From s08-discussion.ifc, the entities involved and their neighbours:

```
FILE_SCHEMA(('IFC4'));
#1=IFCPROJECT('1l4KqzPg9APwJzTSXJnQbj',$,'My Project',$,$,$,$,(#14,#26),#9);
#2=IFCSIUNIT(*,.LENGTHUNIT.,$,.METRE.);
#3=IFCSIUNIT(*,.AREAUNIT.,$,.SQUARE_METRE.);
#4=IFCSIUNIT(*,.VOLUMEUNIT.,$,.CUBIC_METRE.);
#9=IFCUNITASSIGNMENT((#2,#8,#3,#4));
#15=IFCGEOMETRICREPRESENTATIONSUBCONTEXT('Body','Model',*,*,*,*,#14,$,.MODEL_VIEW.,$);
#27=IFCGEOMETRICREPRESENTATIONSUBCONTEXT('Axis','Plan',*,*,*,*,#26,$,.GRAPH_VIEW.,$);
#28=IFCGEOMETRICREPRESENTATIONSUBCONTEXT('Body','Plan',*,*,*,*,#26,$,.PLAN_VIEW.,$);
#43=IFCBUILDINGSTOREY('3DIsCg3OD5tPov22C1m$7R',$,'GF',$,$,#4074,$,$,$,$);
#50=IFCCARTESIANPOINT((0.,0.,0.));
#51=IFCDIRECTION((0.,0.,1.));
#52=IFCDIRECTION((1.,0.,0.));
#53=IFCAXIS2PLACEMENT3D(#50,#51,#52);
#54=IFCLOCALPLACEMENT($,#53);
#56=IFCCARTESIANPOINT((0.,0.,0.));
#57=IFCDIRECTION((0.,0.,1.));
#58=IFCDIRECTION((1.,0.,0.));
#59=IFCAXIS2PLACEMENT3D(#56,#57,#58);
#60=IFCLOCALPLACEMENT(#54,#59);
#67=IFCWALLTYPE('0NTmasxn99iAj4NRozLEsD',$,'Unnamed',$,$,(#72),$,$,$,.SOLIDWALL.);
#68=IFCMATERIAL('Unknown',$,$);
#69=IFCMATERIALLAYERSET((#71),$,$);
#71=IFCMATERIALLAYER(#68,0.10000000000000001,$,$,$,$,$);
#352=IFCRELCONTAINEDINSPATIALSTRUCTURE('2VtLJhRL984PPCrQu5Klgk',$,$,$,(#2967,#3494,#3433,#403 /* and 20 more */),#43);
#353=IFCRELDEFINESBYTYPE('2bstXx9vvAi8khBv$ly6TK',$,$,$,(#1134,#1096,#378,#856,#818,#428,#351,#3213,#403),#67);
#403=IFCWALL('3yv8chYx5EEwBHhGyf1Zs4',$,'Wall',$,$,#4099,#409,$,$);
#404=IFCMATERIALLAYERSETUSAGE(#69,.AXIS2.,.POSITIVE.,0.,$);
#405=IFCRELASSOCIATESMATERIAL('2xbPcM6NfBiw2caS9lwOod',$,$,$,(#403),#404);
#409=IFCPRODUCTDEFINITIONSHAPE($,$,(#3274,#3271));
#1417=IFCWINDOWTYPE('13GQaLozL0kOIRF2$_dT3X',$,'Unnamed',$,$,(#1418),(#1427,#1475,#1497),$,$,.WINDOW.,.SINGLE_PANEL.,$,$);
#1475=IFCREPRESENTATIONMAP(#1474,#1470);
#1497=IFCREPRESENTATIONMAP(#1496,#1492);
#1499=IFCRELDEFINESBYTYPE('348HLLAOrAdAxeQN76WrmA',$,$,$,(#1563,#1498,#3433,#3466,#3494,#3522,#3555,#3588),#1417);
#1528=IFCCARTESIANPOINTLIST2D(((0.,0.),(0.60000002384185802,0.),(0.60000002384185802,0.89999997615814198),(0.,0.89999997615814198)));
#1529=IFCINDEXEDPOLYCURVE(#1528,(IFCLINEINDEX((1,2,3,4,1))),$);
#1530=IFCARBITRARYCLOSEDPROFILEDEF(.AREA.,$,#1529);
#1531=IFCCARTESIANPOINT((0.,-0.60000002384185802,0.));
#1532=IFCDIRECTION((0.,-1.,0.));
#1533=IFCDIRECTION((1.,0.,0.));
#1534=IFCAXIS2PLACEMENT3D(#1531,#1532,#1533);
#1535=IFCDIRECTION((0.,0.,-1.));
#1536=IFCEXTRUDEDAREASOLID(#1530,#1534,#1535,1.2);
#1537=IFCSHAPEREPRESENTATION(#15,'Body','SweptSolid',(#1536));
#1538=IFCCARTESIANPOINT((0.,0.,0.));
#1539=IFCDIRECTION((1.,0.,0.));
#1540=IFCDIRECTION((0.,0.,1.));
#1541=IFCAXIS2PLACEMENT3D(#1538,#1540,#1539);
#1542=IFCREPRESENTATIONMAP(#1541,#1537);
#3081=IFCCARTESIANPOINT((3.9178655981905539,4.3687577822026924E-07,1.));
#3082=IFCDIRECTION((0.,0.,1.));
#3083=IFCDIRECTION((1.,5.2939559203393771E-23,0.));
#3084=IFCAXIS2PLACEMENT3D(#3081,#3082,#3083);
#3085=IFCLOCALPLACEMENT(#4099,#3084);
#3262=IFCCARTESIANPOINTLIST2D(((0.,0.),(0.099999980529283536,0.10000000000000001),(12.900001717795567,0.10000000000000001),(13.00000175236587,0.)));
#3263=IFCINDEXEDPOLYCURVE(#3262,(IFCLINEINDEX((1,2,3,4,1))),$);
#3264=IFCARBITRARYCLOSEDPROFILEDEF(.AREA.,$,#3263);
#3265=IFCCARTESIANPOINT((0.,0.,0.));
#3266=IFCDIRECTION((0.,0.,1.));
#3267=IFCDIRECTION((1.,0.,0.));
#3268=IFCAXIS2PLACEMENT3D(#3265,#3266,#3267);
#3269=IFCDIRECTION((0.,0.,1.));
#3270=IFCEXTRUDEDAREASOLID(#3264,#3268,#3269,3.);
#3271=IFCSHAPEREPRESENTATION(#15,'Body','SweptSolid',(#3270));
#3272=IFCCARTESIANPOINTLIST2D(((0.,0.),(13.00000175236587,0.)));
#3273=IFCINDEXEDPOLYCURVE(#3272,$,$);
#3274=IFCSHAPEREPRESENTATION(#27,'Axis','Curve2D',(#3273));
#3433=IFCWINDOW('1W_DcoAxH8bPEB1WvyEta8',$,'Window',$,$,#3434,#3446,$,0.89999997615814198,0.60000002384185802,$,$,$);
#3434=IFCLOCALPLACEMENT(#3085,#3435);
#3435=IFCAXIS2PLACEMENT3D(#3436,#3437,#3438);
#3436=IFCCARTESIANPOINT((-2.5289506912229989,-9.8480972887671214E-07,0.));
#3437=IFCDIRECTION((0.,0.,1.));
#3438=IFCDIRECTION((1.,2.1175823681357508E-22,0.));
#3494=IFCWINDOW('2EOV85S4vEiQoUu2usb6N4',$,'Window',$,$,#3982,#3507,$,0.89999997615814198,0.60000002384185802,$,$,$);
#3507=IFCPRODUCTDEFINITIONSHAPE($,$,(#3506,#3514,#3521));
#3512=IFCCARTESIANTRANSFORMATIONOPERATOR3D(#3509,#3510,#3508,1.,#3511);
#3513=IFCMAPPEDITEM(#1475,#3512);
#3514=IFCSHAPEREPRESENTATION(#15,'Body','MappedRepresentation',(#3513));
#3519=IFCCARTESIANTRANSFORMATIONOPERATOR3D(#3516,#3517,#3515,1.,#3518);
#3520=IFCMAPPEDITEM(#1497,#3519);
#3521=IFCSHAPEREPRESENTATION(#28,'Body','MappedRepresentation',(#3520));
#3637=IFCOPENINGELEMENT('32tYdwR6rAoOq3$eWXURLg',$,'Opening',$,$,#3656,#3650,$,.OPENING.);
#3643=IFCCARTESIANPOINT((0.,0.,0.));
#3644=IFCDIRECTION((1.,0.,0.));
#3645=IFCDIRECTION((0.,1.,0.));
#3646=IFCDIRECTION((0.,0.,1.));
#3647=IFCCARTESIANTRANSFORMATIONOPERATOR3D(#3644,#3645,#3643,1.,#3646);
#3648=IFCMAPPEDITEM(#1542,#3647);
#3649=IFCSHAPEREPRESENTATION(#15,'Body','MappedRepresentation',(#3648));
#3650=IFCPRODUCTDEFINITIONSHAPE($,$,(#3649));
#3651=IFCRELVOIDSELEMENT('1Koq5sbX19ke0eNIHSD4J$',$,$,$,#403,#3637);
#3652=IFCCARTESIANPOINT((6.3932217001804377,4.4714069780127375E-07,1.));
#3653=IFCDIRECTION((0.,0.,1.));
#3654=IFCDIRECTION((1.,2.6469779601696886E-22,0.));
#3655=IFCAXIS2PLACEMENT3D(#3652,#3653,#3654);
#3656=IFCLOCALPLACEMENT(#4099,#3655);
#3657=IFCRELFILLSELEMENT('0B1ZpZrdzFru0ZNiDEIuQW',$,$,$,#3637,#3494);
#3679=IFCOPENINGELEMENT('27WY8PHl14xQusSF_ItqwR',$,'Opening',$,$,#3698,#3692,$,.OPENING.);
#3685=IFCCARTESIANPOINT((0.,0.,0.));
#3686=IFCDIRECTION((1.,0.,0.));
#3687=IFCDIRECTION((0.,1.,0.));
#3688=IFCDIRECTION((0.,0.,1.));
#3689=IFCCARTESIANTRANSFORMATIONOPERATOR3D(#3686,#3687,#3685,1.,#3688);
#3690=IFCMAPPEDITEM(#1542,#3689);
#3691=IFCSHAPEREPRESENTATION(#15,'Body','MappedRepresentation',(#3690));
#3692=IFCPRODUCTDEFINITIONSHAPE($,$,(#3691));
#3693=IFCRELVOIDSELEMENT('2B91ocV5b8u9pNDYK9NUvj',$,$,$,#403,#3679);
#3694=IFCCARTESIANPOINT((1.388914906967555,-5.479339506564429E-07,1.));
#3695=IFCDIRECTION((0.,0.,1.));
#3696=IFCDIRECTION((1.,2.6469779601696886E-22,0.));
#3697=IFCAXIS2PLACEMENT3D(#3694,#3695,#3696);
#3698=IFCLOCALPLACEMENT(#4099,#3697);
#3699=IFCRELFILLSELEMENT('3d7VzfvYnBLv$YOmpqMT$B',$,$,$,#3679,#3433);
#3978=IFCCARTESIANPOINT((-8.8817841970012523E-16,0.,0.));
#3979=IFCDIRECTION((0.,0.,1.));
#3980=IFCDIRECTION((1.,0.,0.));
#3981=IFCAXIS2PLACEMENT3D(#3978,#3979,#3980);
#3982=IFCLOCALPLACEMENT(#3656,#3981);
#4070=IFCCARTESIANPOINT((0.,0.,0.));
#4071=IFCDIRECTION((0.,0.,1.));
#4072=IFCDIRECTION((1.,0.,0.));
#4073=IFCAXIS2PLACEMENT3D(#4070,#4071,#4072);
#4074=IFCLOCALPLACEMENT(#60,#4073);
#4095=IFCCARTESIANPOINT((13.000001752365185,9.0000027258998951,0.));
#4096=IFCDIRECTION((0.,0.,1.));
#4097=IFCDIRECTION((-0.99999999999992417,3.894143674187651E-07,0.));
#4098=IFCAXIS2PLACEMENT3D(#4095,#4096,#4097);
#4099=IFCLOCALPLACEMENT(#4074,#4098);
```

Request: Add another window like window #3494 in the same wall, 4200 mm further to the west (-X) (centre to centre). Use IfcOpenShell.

```python
import ifcopenshell
import ifcopenshell.api.feature
import ifcopenshell.api.geometry
import ifcopenshell.api.root
import ifcopenshell.geom
import ifcopenshell.util.element
import ifcopenshell.util.placement
import ifcopenshell.util.shape
import ifcopenshell.util.unit

model = ifcopenshell.open("s08-discussion.ifc")
unit_scale = ifcopenshell.util.unit.calculate_unit_scale(model)
settings = ifcopenshell.geom.settings()


def volume(element):
    """Net volume in cubic metres, openings subtracted."""
    shape = ifcopenshell.geom.create_shape(settings, element)
    return ifcopenshell.util.shape.get_volume(shape.geometry)


window = model.by_id(3494)
opening = window.FillsVoids[0].RelatingOpeningElement
wall = opening.VoidsElements[0].RelatingBuildingElement
before = volume(wall)
shift = ifcopenshell.util.placement.get_local_placement(wall.ObjectPlacement)[:3, 0] * 4.2 / unit_scale

# copy_class copies the void relationship, type, container and properties, but no geometry.
new_opening = ifcopenshell.api.root.copy_class(model, product=opening)
new_opening.Representation = ifcopenshell.util.element.copy_deep(
    model, opening.Representation, exclude=["IfcGeometricRepresentationContext", "IfcRepresentationMap"]
)
new_window = ifcopenshell.api.root.copy_class(model, product=window)
new_window.Representation = ifcopenshell.util.element.copy_deep(
    model, window.Representation, exclude=["IfcGeometricRepresentationContext", "IfcRepresentationMap"]
)
ifcopenshell.api.feature.add_filling(model, opening=new_opening, element=new_window)

for old, new in ((opening, new_opening), (window, new_window)):
    matrix = ifcopenshell.util.placement.get_local_placement(old.ObjectPlacement)
    matrix[:3, 3] += shift
    ifcopenshell.api.geometry.edit_object_placement(model, product=new, matrix=matrix, is_si=False)

after = volume(wall)

print(f"wall volume {before:.3f} -> {after:.3f} m3")

model.write("s08-discussion_updated.ifc")
```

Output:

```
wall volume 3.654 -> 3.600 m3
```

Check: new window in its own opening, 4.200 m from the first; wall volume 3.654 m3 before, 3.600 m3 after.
